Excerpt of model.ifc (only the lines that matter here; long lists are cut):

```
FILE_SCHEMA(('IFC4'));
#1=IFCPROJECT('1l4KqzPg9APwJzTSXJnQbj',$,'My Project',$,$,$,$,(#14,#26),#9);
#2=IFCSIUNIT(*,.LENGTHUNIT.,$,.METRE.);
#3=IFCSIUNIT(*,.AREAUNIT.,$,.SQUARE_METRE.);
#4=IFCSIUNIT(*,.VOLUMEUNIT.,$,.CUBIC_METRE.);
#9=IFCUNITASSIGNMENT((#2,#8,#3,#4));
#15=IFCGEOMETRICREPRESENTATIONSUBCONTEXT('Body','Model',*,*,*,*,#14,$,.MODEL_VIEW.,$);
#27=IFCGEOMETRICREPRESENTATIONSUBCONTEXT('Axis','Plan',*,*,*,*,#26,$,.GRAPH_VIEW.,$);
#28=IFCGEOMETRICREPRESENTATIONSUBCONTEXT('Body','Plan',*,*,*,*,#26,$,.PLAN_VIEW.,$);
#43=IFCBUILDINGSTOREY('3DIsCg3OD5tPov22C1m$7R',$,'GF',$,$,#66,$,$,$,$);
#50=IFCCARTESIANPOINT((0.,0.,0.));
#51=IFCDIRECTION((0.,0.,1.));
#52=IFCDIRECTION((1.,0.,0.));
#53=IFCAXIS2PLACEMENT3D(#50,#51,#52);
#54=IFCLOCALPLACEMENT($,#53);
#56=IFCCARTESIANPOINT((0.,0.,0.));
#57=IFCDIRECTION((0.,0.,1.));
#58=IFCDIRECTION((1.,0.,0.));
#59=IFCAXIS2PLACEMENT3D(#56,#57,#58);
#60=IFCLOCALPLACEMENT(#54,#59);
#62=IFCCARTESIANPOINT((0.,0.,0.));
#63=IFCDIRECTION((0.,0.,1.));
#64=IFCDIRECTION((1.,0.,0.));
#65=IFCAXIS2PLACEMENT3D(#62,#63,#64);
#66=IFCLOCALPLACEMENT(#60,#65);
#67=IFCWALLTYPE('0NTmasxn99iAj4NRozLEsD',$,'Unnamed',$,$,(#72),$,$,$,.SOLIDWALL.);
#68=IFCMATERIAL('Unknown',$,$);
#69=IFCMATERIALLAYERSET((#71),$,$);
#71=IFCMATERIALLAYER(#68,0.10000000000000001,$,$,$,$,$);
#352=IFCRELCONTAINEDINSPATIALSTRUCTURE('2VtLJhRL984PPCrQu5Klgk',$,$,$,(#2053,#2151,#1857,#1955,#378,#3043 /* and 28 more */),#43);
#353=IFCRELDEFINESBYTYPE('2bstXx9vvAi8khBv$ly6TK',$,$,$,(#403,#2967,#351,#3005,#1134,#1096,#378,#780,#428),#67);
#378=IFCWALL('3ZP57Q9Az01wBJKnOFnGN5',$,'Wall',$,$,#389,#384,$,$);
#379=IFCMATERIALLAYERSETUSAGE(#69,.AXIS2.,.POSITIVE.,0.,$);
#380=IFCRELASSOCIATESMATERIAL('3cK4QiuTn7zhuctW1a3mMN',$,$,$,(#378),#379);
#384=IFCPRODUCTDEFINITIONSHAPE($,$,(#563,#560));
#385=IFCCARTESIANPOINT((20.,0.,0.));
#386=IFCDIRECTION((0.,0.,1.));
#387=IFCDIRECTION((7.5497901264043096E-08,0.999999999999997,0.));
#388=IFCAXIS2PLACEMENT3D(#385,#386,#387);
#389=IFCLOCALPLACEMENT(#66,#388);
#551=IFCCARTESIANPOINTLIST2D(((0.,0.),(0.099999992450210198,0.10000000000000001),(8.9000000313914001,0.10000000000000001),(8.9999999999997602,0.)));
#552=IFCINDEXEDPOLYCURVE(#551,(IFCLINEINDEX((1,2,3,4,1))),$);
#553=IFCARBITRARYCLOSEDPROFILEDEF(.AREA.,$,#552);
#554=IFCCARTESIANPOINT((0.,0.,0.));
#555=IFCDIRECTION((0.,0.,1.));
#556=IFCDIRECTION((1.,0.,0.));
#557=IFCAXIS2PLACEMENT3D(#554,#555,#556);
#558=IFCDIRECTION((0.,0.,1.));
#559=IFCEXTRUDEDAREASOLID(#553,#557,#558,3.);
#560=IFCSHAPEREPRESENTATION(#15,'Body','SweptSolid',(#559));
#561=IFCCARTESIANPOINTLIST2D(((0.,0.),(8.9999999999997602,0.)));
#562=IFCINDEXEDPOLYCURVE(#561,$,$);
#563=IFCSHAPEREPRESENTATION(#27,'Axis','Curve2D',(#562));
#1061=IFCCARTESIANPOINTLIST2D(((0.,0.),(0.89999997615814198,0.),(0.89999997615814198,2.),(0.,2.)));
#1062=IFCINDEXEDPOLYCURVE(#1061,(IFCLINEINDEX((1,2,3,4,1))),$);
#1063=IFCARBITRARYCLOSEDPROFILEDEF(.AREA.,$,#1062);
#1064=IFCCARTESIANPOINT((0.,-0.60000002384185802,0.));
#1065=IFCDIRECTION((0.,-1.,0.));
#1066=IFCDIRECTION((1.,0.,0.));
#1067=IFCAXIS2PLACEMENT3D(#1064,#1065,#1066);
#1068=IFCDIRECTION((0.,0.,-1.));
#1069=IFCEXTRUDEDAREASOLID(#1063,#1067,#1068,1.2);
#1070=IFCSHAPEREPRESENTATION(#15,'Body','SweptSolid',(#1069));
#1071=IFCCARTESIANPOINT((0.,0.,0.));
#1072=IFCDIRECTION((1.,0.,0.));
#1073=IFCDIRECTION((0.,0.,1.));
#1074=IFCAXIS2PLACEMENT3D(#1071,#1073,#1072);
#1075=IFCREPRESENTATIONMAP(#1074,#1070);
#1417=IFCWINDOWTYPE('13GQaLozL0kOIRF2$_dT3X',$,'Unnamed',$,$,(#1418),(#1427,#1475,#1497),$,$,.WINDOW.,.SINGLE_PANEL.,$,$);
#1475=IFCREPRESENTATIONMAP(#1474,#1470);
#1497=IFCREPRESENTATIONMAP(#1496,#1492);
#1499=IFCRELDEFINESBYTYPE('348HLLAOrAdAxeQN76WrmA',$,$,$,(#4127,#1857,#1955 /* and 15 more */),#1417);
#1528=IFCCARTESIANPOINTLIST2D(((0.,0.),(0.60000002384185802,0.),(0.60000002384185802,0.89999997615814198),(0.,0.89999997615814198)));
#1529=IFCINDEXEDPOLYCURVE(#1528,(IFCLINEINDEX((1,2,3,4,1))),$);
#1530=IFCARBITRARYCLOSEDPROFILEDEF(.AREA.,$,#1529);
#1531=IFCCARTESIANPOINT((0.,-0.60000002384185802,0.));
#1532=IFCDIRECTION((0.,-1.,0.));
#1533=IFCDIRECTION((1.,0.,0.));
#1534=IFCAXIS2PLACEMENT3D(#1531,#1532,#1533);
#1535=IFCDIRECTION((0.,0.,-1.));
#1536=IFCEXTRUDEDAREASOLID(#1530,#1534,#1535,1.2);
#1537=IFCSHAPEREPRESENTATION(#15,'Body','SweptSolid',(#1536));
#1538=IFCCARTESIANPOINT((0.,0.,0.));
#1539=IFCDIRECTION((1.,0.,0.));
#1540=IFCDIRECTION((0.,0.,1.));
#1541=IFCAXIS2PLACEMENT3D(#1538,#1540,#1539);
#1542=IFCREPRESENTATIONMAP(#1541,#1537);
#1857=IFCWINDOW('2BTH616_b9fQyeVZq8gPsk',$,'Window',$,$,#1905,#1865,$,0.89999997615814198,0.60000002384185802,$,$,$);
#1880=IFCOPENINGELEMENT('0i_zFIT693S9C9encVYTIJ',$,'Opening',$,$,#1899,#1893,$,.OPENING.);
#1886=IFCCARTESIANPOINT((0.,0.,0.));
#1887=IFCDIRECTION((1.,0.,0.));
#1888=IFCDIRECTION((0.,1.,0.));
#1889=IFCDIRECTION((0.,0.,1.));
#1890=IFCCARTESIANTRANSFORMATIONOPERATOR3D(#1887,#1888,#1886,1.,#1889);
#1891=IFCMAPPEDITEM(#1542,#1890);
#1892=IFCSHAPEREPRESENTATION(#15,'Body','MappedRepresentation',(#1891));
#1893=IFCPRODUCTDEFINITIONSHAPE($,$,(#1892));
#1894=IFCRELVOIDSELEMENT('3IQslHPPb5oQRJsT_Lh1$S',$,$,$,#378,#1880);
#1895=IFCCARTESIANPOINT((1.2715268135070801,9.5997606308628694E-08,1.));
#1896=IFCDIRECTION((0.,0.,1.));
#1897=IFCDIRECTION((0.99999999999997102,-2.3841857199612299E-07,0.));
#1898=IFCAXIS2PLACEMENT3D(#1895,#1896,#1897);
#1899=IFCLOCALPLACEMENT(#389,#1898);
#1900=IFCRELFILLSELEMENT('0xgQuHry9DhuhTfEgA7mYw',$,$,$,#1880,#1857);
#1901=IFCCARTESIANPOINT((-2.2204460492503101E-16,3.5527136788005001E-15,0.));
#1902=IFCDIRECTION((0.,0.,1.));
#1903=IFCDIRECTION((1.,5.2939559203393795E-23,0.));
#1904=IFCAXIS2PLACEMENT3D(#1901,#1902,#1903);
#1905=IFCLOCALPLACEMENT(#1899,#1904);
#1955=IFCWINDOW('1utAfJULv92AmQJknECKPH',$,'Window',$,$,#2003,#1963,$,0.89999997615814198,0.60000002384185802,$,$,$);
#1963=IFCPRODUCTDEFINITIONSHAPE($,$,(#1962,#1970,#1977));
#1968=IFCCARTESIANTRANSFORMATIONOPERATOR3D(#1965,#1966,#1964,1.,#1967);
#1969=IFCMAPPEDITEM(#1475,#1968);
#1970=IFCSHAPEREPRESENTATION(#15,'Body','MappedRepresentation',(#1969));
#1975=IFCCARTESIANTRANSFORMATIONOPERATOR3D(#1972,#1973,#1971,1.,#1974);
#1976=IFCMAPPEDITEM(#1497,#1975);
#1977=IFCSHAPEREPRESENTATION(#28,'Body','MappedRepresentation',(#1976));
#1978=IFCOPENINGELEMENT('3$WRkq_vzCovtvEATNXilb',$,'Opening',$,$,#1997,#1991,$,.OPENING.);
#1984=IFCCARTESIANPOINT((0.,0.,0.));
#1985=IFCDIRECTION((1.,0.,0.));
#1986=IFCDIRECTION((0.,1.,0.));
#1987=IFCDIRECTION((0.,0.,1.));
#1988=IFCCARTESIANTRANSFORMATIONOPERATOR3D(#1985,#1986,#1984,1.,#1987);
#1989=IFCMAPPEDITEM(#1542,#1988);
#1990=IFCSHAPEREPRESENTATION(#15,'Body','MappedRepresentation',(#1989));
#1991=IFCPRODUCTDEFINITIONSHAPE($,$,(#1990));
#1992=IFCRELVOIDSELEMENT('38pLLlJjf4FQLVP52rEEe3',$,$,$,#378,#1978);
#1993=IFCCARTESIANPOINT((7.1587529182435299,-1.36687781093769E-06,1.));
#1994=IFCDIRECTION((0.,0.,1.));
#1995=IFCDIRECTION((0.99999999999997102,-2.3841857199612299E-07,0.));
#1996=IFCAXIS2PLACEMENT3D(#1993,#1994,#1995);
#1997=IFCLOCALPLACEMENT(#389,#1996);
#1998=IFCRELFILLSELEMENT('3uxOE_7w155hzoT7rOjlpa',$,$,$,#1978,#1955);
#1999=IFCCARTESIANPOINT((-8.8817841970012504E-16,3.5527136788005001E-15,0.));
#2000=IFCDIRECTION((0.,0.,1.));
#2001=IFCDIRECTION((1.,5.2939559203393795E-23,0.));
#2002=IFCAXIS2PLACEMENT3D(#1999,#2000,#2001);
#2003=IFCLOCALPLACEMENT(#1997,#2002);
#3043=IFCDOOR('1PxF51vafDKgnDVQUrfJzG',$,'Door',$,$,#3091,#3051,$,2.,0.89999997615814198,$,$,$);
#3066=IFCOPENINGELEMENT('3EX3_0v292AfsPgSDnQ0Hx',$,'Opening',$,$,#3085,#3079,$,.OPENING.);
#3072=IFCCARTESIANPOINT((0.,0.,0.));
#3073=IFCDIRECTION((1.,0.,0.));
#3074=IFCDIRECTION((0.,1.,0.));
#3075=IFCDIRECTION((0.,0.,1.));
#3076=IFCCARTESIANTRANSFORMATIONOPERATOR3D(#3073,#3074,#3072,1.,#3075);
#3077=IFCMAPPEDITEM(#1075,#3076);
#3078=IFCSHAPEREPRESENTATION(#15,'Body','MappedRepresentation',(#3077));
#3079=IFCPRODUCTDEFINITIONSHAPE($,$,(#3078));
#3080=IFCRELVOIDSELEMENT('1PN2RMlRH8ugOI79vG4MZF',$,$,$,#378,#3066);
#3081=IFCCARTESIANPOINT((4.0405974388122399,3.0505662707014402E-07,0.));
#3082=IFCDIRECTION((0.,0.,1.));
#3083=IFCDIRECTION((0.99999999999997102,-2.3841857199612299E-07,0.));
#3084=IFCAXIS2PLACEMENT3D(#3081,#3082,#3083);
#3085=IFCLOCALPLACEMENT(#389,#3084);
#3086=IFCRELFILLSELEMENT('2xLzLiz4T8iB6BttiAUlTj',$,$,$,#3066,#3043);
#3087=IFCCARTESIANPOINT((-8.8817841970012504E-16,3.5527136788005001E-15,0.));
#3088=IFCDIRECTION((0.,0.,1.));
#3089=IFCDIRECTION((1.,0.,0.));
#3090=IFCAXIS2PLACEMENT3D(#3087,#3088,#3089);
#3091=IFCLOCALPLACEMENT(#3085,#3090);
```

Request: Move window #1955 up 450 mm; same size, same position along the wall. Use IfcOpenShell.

```python
import numpy as np
import ifcopenshell
import ifcopenshell.api.geometry
import ifcopenshell.util.placement
import ifcopenshell.util.unit

model = ifcopenshell.open("model.ifc")
unit_scale = ifcopenshell.util.unit.calculate_unit_scale(model)

window = model.by_id(1955)
opening = window.FillsVoids[0].RelatingOpeningElement
dz = 0.45

shift = np.array([0.0, 0.0, dz])
# The window is placed relative to its opening, so it follows when the opening moves.
matrix = ifcopenshell.util.placement.get_local_placement(opening.ObjectPlacement)
matrix[:3, 3] += shift
ifcopenshell.api.geometry.edit_object_placement(
    model, product=opening, matrix=matrix, is_si=False, should_transform_children=True
)

print(f"moved by {dz * unit_scale:+.3f} m")

model.write("model_updated.ifc")
```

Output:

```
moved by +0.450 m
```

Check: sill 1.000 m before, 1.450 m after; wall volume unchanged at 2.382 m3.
